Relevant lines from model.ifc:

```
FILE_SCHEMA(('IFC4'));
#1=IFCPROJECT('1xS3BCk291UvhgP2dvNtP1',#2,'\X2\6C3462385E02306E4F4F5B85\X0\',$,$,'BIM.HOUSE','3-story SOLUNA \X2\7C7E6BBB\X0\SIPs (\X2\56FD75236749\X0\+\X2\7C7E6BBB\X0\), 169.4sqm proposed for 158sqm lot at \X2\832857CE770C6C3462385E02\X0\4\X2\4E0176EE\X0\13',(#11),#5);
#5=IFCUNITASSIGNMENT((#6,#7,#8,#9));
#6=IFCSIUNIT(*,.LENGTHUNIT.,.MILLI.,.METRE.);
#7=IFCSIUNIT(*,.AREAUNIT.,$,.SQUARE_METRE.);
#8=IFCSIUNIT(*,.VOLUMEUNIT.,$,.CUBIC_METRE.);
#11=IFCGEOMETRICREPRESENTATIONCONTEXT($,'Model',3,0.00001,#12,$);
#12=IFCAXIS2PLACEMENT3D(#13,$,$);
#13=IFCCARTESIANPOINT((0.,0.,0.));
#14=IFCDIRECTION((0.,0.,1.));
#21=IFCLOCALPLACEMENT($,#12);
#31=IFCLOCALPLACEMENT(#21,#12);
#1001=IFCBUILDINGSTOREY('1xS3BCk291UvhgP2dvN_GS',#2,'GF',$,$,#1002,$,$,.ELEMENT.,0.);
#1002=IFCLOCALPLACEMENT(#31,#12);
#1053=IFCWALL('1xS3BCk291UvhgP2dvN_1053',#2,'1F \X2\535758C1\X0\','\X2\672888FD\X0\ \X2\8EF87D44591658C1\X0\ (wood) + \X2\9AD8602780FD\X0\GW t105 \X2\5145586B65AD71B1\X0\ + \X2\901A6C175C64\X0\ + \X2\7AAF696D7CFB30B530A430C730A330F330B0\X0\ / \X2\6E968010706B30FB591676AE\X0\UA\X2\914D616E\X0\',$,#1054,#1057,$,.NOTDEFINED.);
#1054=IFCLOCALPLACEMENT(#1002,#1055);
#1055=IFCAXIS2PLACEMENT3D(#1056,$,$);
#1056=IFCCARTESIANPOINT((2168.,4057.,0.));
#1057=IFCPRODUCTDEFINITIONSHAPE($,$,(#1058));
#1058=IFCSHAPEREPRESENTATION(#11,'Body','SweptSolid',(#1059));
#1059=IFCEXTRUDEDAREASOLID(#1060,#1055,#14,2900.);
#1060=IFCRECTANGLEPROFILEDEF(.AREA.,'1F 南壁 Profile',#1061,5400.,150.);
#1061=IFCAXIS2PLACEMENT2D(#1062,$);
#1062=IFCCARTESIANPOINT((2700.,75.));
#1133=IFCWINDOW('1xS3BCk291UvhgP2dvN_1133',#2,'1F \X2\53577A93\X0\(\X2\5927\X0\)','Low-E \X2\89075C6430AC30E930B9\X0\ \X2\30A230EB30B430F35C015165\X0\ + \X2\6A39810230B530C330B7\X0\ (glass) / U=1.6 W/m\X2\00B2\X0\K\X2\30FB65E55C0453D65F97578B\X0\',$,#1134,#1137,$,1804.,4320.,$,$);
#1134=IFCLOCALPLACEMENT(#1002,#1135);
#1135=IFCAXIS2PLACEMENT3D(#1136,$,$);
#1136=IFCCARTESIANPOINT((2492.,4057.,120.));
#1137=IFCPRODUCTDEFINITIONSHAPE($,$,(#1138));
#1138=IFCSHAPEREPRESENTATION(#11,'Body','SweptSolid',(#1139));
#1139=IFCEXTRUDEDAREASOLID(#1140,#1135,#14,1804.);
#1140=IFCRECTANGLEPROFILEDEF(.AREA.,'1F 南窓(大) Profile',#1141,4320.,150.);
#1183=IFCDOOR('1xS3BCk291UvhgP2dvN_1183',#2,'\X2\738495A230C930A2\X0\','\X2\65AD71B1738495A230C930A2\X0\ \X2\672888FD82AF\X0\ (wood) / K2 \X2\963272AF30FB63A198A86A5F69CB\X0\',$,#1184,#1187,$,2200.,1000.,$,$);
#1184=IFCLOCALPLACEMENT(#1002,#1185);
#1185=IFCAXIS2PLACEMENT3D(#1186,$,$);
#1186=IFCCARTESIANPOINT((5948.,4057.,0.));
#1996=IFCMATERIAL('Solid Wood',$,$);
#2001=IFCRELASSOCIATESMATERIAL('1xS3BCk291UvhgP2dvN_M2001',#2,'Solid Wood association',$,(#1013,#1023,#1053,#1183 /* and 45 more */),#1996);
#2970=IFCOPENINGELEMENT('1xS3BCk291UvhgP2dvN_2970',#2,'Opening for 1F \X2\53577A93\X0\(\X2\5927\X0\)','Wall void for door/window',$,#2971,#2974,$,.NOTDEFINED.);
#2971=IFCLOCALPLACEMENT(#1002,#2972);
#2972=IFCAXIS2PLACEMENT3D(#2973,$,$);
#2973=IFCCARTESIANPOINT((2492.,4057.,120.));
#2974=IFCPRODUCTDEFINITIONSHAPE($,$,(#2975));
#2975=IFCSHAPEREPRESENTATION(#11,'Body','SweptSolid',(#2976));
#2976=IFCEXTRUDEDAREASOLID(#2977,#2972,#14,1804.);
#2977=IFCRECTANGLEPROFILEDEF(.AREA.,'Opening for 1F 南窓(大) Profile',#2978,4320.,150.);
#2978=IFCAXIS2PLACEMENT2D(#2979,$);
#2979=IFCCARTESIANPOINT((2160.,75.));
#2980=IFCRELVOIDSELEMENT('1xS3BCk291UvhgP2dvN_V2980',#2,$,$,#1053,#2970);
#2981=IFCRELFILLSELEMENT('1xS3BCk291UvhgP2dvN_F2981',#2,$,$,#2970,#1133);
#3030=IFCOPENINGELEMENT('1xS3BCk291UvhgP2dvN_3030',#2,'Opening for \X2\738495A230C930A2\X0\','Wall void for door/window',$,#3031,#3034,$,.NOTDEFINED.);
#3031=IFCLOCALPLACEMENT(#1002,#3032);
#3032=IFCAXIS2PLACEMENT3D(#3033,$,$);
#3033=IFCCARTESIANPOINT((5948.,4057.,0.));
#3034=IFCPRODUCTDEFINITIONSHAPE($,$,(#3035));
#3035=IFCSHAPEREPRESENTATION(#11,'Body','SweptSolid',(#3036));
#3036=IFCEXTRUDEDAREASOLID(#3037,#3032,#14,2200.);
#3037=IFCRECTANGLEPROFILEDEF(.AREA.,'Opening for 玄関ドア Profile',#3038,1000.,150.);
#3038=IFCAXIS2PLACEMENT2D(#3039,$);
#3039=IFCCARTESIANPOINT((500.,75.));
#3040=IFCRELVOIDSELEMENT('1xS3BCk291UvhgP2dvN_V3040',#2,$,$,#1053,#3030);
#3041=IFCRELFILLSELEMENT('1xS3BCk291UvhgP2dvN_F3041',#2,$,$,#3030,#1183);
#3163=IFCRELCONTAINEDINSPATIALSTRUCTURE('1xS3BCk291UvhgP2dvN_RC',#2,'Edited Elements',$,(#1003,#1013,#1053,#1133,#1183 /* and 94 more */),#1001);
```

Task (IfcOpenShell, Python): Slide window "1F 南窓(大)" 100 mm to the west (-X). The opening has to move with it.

```python
import ifcopenshell
import ifcopenshell.api.geometry
import ifcopenshell.util.placement
import ifcopenshell.util.unit

model = ifcopenshell.open("model.ifc")
unit_scale = ifcopenshell.util.unit.calculate_unit_scale(model)

window = model.by_guid("1xS3BCk291UvhgP2dvN_1133")
opening = window.FillsVoids[0].RelatingOpeningElement
wall = opening.VoidsElements[0].RelatingBuildingElement

wall_matrix = ifcopenshell.util.placement.get_local_placement(wall.ObjectPlacement)
shift = wall_matrix[:3, 0] * -0.1 / unit_scale
before = ifcopenshell.util.placement.get_local_placement(window.ObjectPlacement)[:3, 3].copy()

# The window is not placed relative to its opening, so move both.
for product in (opening, window):
    matrix = ifcopenshell.util.placement.get_local_placement(product.ObjectPlacement)
    matrix[:3, 3] += shift
    ifcopenshell.api.geometry.edit_object_placement(model, product=product, matrix=matrix, is_si=False)

after = ifcopenshell.util.placement.get_local_placement(window.ObjectPlacement)[:3, 3]
print("window moved by", (after - before).round(3) + 0.0)

model.write("model_edited.ifc")
```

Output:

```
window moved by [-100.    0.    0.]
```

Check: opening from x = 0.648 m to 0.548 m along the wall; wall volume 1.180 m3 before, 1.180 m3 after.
